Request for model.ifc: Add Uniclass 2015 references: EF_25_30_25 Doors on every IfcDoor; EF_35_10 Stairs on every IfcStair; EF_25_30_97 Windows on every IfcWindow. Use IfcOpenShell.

First a look at what the model holds.

```python
import ifcopenshell

model = ifcopenshell.open("model.ifc")
print(model.schema)
print("classifications:", [c.Name for c in model.by_type("IfcClassification")])
for ifc_class in ("IfcDoor", "IfcRoof", "IfcStair", "IfcWall", "IfcWindow"):
    print(ifc_class, len(model.by_type(ifc_class)))
```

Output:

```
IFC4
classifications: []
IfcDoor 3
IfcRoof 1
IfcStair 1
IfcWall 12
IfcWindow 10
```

```python
import ifcopenshell
import ifcopenshell.api.classification

model = ifcopenshell.open("model.ifc")

system = ifcopenshell.api.classification.add_classification(model, classification="Uniclass 2015")

codes = {
    "IfcDoor": ("EF_25_30_25", "Doors"),
    "IfcStair": ("EF_35_10", "Stairs"),
    "IfcWindow": ("EF_25_30_97", "Windows"),
}
for ifc_class, (code, name) in codes.items():
    products = model.by_type(ifc_class)
    ifcopenshell.api.classification.add_reference(
        model, products=products, classification=system, identification=code, name=name
    )
    print(code, len(products))

model.write("model_v2.ifc")
```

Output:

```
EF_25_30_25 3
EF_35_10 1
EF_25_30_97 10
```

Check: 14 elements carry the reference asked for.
